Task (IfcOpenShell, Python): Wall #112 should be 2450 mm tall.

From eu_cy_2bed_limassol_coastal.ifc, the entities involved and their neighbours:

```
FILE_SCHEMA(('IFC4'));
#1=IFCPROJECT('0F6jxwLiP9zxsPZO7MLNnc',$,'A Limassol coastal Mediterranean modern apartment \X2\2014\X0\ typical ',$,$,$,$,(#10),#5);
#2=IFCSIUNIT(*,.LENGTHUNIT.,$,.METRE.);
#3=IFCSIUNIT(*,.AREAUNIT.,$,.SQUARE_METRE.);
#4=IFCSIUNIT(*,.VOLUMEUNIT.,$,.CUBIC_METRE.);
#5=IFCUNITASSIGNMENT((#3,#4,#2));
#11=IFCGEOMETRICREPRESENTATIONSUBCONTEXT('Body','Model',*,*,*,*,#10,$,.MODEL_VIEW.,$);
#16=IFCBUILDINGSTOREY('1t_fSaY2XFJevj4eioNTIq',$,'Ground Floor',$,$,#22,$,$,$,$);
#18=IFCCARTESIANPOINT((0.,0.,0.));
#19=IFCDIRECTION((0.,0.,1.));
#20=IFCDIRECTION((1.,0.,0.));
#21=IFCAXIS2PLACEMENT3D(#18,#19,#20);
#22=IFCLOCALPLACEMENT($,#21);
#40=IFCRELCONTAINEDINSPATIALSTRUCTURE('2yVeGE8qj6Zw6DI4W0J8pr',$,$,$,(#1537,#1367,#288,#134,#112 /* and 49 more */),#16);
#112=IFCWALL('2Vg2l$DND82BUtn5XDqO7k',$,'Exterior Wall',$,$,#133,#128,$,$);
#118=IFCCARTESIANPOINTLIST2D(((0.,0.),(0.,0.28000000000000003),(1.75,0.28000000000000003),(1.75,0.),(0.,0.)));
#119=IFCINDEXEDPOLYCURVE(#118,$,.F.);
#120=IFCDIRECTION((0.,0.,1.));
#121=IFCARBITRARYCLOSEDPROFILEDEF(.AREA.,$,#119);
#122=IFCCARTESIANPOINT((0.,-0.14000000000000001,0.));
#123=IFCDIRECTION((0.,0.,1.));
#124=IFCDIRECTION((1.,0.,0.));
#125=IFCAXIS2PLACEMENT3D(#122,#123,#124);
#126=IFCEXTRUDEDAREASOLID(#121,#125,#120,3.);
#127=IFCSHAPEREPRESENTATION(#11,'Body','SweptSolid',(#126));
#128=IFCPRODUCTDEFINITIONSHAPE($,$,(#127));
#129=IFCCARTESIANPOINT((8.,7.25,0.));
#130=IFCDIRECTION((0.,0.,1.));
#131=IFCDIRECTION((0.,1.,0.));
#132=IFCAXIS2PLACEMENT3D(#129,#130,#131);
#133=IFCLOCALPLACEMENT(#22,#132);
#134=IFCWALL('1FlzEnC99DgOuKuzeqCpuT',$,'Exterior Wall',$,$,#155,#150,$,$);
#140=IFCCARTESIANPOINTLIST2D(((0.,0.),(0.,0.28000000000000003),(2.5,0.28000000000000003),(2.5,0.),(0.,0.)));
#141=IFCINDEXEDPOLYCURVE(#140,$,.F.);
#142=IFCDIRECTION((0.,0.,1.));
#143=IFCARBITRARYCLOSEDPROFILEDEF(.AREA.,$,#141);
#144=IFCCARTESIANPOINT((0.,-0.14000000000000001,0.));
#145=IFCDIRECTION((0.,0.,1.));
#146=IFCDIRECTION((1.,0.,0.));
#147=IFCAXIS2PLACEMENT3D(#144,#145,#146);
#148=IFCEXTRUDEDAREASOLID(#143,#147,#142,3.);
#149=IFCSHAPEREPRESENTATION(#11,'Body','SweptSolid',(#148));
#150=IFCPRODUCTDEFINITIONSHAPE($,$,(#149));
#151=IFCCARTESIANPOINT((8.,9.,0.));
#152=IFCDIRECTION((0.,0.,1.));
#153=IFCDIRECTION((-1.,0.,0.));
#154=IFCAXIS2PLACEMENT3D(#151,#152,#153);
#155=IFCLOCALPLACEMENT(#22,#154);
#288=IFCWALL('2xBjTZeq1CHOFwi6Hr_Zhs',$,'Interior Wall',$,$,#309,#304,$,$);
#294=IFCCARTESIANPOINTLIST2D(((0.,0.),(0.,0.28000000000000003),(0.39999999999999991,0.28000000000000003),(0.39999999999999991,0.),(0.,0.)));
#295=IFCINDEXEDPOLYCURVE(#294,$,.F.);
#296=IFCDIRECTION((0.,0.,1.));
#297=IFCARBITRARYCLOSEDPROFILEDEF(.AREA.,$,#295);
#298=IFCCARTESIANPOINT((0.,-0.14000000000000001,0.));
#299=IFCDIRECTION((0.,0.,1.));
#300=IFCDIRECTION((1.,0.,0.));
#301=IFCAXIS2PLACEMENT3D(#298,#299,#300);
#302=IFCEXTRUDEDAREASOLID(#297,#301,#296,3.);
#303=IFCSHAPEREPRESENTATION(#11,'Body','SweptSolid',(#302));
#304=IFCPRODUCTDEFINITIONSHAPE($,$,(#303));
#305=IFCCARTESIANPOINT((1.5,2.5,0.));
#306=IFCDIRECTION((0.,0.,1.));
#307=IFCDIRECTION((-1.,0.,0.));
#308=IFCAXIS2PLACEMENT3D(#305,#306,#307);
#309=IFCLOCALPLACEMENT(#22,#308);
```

```python
import ifcopenshell
import ifcopenshell.geom
import ifcopenshell.util.representation
import ifcopenshell.util.shape
import ifcopenshell.util.unit

model = ifcopenshell.open("eu_cy_2bed_limassol_coastal.ifc")
unit_scale = ifcopenshell.util.unit.calculate_unit_scale(model)
settings = ifcopenshell.geom.settings()


def volume(element):
    """Net volume in cubic metres, openings subtracted."""
    shape = ifcopenshell.geom.create_shape(settings, element)
    return ifcopenshell.util.shape.get_volume(shape.geometry)


wall = model.by_guid("2Vg2l$DND82BUtn5XDqO7k")
before = volume(wall)

body = ifcopenshell.util.representation.get_representation(wall, "Model", "Body")
solid = body.Items[0]
old_height = solid.Depth
solid.Depth = 2.45 / unit_scale
after = volume(wall)

print(f"height {old_height:g} -> {solid.Depth:g}, volume {before:.3f} -> {after:.3f} m3")

model.write("eu_cy_2bed_limassol_coastal_rev.ifc")
```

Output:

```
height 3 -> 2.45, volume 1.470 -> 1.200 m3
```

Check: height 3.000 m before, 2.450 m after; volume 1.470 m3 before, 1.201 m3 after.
